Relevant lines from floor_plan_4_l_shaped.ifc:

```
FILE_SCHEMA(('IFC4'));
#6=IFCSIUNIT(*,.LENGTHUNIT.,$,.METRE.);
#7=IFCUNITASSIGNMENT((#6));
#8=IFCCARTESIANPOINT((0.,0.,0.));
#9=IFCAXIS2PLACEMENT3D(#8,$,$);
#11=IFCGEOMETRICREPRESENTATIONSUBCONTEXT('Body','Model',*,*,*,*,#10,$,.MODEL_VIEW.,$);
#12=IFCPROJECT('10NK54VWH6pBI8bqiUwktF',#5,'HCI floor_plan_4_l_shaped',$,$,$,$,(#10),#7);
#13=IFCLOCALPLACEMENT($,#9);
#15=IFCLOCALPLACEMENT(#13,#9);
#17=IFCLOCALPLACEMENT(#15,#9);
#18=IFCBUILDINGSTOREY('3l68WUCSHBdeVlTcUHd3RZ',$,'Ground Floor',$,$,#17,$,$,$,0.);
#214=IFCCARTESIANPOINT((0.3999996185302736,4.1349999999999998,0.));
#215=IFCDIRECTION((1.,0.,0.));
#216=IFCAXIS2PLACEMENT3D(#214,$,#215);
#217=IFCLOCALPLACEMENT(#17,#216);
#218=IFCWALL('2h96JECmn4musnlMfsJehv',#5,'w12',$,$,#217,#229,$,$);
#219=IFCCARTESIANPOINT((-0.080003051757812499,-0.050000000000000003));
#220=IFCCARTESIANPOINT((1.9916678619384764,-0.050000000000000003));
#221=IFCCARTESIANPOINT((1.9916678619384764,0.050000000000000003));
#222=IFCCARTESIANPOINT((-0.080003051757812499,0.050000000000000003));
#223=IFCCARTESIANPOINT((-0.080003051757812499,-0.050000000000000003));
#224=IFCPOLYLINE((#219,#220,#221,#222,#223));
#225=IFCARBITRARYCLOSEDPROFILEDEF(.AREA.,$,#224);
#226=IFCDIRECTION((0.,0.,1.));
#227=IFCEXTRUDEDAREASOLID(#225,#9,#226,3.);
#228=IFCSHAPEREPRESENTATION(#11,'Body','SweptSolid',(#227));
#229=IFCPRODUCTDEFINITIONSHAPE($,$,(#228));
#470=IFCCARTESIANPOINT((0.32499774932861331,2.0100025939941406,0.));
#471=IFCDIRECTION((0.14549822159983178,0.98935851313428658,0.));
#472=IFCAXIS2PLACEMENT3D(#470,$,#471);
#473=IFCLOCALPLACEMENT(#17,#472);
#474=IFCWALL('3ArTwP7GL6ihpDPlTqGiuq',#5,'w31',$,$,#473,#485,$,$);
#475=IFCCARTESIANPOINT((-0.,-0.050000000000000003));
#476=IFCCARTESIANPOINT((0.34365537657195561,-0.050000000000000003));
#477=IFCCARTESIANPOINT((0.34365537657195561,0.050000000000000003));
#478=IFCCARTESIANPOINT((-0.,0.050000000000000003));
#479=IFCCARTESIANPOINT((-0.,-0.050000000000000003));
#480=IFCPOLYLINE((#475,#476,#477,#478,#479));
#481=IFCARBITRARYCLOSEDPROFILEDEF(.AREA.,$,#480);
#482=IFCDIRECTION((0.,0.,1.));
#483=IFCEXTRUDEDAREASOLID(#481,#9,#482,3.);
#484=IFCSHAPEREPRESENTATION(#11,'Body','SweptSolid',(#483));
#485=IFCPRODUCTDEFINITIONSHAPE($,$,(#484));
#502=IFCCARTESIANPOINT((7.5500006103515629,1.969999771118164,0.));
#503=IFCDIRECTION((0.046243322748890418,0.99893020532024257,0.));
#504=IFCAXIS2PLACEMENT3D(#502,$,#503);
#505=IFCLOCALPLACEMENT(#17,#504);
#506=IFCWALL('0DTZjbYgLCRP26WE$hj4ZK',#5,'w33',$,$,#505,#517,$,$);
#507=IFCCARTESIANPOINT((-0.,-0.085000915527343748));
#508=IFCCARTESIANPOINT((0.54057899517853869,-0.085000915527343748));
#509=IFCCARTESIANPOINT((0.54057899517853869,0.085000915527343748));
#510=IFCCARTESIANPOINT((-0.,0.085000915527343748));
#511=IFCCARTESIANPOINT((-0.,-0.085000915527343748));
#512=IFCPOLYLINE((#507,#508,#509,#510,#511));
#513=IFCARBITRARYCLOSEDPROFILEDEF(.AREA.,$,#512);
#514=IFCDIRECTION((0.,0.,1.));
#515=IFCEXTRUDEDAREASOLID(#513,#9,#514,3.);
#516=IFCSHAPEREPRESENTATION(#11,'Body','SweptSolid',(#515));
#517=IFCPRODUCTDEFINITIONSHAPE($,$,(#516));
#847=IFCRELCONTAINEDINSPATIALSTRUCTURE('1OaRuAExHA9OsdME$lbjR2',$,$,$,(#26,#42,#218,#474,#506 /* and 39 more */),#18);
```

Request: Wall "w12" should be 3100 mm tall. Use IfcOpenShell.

```python
import ifcopenshell
import ifcopenshell.geom
import ifcopenshell.util.representation
import ifcopenshell.util.shape

model = ifcopenshell.open("floor_plan_4_l_shaped.ifc")
settings = ifcopenshell.geom.settings()


def volume(element):
    """Net volume in cubic metres, openings subtracted."""
    shape = ifcopenshell.geom.create_shape(settings, element)
    return ifcopenshell.util.shape.get_volume(shape.geometry)


wall = model.by_guid("2h96JECmn4musnlMfsJehv")
before = volume(wall)

body = ifcopenshell.util.representation.get_representation(wall, "Model", "Body")
solid = body.Items[0]
old_height = solid.Depth
solid.Depth = 3.1
after = volume(wall)

print(f"height {old_height:g} -> {solid.Depth:g}, volume {before:.3f} -> {after:.3f} m3")

model.write("floor_plan_4_l_shaped_v2.ifc")
```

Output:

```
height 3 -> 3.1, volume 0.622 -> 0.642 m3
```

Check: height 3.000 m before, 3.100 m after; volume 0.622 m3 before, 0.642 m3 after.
